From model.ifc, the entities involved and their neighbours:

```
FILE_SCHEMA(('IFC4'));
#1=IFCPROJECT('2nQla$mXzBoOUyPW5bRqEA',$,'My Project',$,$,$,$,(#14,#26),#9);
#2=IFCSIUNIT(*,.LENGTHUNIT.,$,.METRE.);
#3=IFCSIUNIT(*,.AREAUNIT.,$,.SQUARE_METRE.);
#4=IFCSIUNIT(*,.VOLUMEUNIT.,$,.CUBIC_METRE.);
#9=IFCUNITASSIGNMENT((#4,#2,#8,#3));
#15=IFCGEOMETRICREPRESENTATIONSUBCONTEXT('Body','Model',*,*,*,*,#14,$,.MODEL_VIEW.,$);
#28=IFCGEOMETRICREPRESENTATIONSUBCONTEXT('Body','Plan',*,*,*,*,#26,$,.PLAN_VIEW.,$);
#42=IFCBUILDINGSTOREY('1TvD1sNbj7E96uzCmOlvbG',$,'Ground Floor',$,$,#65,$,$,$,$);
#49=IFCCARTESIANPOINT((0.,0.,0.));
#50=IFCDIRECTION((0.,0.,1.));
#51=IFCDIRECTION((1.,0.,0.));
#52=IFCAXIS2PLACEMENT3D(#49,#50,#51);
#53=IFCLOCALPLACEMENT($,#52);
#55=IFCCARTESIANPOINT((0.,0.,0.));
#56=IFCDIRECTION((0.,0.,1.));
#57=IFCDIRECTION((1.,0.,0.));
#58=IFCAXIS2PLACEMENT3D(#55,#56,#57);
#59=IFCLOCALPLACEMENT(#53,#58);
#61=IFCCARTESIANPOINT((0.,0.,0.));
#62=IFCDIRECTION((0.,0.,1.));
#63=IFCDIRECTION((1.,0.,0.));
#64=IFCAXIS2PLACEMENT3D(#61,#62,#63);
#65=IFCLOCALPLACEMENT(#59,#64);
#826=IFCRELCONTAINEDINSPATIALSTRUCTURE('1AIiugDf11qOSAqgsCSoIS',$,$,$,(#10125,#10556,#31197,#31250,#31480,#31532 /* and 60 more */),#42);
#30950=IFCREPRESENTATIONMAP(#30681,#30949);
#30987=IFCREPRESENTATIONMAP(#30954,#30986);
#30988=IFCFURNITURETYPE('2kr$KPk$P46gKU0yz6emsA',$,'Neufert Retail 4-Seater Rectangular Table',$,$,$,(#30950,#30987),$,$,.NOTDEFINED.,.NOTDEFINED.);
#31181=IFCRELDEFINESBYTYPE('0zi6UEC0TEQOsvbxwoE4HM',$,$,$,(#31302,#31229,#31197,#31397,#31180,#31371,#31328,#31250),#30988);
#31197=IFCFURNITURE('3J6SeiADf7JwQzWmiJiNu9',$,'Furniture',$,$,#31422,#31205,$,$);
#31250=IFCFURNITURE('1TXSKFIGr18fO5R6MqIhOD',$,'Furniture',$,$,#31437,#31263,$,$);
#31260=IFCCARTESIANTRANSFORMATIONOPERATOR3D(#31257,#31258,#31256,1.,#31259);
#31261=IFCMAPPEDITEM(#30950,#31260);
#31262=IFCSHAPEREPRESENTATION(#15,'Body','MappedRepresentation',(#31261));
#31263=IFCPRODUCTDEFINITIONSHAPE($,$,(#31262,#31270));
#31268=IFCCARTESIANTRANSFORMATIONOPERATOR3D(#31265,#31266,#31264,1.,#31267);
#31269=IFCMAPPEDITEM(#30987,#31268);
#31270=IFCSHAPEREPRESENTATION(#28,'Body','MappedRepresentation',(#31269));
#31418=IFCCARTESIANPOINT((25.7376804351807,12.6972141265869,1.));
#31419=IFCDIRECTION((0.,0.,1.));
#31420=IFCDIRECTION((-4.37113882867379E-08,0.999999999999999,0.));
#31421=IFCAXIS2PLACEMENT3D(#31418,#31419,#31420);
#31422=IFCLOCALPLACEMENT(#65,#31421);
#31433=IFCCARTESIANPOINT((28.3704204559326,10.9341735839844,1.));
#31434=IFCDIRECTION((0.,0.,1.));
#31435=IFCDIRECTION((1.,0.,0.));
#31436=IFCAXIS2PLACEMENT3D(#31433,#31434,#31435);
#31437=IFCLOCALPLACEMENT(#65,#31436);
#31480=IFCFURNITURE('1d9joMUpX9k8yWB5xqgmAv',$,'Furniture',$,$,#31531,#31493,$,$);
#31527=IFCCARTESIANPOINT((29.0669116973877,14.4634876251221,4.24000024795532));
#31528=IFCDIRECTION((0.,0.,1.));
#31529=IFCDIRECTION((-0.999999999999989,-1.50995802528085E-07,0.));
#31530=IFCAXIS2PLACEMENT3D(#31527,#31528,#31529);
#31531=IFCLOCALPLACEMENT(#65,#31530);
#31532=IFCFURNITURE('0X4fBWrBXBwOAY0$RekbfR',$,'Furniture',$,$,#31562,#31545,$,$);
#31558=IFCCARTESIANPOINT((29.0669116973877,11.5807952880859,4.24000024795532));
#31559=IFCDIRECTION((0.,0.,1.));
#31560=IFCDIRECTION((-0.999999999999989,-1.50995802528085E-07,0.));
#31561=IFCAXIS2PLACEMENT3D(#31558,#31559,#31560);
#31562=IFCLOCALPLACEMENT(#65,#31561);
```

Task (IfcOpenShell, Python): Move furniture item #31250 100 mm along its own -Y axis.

```python
import ifcopenshell
import ifcopenshell.api.geometry
import ifcopenshell.util.placement

model = ifcopenshell.open("model.ifc")

item = model.by_id(31250)
matrix = ifcopenshell.util.placement.get_local_placement(item.ObjectPlacement)
matrix[:3, 3] -= matrix[:3, 1] * 0.1
ifcopenshell.api.geometry.edit_object_placement(model, product=item, matrix=matrix, is_si=False)

print(ifcopenshell.util.placement.get_local_placement(item.ObjectPlacement).round(3) + 0.0)

model.write("model_updated.ifc")
```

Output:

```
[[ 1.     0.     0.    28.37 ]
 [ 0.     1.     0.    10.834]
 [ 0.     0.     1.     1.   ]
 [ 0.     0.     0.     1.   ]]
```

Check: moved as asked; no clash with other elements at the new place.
